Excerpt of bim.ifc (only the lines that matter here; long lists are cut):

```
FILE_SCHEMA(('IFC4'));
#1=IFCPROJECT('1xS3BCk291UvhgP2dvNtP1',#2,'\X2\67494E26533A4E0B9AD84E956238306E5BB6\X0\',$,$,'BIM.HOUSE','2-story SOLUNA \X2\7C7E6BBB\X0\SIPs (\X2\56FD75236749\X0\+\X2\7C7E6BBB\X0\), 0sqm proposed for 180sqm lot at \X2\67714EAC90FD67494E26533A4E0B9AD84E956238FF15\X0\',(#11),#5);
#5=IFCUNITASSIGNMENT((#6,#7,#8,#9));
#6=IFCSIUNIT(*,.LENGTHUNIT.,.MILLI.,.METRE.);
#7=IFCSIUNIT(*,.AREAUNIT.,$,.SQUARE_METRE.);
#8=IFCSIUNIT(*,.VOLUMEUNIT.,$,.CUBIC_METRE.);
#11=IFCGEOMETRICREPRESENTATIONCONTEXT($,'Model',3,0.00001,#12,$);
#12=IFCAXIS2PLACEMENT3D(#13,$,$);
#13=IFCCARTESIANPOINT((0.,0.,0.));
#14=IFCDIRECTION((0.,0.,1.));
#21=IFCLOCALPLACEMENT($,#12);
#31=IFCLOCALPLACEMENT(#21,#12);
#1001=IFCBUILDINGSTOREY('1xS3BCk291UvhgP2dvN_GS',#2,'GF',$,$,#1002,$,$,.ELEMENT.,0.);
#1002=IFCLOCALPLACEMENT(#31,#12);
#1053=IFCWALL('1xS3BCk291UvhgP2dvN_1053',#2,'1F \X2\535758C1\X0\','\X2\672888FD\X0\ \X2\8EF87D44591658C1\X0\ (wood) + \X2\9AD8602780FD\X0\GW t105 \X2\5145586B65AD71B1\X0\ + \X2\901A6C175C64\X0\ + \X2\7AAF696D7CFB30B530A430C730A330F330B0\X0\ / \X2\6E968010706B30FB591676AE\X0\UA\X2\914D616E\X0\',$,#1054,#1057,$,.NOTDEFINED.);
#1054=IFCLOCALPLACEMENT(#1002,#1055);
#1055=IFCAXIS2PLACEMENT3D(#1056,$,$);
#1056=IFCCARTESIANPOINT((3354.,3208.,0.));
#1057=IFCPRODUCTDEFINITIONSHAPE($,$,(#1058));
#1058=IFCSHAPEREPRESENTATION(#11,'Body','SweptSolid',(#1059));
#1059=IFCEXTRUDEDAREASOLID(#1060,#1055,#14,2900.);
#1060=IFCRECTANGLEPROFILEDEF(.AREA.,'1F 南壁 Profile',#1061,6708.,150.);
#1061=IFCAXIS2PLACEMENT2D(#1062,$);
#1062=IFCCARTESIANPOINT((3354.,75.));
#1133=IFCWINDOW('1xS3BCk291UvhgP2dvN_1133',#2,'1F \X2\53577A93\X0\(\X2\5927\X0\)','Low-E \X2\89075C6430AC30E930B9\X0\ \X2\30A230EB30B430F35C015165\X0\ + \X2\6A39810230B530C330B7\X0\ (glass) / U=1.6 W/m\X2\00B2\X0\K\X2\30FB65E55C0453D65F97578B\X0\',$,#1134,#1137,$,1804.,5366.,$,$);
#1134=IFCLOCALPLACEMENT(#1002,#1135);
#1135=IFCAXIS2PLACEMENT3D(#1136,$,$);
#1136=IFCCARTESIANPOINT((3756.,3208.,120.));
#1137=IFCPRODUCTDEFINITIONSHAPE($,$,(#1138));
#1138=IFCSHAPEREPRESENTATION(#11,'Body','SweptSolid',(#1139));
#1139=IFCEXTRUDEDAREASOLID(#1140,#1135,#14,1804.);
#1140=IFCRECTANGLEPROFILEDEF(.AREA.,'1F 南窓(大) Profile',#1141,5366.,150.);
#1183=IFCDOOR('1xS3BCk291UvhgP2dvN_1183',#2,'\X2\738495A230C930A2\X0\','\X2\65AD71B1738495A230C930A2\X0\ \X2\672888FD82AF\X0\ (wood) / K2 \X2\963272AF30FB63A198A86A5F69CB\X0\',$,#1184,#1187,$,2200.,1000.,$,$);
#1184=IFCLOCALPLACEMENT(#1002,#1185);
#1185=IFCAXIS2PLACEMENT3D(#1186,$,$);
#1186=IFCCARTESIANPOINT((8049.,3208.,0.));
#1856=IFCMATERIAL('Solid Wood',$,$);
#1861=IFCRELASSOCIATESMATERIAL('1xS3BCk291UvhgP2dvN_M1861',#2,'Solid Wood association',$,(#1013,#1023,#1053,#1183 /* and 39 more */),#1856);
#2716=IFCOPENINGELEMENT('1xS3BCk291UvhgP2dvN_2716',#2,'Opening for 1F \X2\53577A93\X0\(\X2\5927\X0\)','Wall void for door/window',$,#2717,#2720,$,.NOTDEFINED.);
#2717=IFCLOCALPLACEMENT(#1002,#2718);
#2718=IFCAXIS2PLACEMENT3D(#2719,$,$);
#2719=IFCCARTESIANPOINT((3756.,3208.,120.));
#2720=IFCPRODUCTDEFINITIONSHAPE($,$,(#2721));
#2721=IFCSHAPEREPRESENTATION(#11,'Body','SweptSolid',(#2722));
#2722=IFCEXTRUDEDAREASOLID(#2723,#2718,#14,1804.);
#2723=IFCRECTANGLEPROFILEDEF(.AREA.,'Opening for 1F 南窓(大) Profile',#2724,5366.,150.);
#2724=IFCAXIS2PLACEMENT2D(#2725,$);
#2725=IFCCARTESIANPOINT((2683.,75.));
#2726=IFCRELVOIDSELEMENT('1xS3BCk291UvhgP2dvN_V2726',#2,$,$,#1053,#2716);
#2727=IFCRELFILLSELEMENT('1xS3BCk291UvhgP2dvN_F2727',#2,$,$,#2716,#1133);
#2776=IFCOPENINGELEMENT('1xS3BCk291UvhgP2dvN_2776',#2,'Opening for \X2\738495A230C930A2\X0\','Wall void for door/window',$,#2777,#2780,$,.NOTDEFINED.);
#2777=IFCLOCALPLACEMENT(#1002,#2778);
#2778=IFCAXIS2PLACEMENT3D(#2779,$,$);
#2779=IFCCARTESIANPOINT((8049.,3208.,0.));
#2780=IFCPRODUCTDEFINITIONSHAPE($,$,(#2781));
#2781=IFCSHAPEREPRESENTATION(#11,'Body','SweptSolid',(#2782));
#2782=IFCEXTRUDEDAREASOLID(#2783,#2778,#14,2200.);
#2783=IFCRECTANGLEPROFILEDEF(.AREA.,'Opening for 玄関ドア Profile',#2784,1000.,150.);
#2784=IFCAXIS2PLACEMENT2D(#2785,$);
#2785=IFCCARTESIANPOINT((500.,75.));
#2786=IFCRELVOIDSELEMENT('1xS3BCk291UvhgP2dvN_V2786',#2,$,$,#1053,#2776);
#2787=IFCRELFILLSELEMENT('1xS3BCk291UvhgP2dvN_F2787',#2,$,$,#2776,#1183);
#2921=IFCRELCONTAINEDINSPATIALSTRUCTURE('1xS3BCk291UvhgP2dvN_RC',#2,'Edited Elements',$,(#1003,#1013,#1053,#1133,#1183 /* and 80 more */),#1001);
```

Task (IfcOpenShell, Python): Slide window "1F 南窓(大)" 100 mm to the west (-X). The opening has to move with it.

```python
import ifcopenshell
import ifcopenshell.api.geometry
import ifcopenshell.util.placement
import ifcopenshell.util.unit

model = ifcopenshell.open("bim.ifc")
unit_scale = ifcopenshell.util.unit.calculate_unit_scale(model)

window = model.by_guid("1xS3BCk291UvhgP2dvN_1133")
opening = window.FillsVoids[0].RelatingOpeningElement
wall = opening.VoidsElements[0].RelatingBuildingElement

wall_matrix = ifcopenshell.util.placement.get_local_placement(wall.ObjectPlacement)
shift = wall_matrix[:3, 0] * -0.1 / unit_scale
before = ifcopenshell.util.placement.get_local_placement(window.ObjectPlacement)[:3, 3].copy()

# The window is not placed relative to its opening, so move both.
for product in (opening, window):
    matrix = ifcopenshell.util.placement.get_local_placement(product.ObjectPlacement)
    matrix[:3, 3] += shift
    ifcopenshell.api.geometry.edit_object_placement(model, product=product, matrix=matrix, is_si=False)

after = ifcopenshell.util.placement.get_local_placement(window.ObjectPlacement)[:3, 3]
print("window moved by", (after - before).round(3) + 0.0)

model.write("bim_rev.ifc")
```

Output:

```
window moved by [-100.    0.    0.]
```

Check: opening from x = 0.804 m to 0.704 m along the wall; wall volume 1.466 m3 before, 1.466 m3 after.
